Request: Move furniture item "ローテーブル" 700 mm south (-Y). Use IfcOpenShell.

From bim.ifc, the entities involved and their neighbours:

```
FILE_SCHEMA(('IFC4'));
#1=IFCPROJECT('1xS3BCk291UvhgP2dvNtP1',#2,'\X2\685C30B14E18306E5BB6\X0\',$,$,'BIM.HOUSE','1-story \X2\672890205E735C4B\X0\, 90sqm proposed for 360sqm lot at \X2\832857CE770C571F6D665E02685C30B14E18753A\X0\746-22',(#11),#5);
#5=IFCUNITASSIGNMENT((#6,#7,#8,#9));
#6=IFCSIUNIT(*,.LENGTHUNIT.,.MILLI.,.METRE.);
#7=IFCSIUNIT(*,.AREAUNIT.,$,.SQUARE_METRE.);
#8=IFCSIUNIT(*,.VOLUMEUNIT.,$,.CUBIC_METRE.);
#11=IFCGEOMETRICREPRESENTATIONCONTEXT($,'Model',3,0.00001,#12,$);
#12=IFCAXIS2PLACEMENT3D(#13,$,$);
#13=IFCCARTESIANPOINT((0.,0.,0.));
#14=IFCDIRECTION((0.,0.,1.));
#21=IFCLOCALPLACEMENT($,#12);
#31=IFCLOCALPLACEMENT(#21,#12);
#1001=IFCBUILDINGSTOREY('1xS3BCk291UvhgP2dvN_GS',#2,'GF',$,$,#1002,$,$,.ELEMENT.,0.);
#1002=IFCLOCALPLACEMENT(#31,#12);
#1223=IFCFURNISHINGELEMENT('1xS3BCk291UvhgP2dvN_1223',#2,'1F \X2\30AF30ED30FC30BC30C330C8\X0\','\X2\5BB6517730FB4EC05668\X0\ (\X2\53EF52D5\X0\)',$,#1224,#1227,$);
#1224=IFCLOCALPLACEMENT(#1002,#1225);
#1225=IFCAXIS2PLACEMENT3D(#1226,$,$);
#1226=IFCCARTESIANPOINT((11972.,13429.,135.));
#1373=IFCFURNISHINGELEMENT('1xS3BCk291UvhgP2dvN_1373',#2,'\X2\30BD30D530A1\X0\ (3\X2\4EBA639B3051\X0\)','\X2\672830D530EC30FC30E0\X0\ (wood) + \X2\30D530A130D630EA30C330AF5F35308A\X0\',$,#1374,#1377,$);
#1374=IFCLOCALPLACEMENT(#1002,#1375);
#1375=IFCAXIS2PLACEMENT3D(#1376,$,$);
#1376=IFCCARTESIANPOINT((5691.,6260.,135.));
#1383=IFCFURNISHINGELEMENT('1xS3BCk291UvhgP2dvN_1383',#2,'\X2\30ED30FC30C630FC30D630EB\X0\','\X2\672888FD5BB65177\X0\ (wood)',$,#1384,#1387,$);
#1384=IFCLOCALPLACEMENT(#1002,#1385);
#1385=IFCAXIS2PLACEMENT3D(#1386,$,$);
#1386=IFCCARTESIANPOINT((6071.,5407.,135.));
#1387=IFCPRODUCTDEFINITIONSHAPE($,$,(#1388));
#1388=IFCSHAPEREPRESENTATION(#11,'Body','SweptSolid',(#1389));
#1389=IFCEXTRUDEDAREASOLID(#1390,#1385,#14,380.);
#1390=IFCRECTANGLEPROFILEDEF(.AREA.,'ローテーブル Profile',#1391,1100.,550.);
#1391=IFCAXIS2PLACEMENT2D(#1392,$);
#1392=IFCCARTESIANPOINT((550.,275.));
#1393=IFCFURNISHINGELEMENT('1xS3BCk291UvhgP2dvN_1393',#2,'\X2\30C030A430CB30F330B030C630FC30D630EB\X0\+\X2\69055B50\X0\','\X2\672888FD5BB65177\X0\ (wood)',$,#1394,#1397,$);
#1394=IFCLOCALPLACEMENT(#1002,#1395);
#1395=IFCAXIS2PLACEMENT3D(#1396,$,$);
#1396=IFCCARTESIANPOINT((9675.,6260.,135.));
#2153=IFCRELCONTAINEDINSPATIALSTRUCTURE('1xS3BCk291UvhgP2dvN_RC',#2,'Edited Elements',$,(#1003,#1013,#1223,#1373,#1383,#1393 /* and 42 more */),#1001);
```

```python
import ifcopenshell
import ifcopenshell.api.geometry
import ifcopenshell.util.placement
import ifcopenshell.util.unit

model = ifcopenshell.open("bim.ifc")
unit_scale = ifcopenshell.util.unit.calculate_unit_scale(model)

item = model.by_guid("1xS3BCk291UvhgP2dvN_1383")
matrix = ifcopenshell.util.placement.get_local_placement(item.ObjectPlacement)
matrix[1, 3] -= 0.7 / unit_scale
ifcopenshell.api.geometry.edit_object_placement(model, product=item, matrix=matrix, is_si=False)

print(ifcopenshell.util.placement.get_local_placement(item.ObjectPlacement).round(3) + 0.0)

model.write("bim-out.ifc")
```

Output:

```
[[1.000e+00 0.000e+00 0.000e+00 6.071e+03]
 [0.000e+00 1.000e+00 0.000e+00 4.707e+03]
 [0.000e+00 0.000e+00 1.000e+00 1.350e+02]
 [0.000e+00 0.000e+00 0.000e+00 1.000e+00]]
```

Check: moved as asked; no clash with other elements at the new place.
